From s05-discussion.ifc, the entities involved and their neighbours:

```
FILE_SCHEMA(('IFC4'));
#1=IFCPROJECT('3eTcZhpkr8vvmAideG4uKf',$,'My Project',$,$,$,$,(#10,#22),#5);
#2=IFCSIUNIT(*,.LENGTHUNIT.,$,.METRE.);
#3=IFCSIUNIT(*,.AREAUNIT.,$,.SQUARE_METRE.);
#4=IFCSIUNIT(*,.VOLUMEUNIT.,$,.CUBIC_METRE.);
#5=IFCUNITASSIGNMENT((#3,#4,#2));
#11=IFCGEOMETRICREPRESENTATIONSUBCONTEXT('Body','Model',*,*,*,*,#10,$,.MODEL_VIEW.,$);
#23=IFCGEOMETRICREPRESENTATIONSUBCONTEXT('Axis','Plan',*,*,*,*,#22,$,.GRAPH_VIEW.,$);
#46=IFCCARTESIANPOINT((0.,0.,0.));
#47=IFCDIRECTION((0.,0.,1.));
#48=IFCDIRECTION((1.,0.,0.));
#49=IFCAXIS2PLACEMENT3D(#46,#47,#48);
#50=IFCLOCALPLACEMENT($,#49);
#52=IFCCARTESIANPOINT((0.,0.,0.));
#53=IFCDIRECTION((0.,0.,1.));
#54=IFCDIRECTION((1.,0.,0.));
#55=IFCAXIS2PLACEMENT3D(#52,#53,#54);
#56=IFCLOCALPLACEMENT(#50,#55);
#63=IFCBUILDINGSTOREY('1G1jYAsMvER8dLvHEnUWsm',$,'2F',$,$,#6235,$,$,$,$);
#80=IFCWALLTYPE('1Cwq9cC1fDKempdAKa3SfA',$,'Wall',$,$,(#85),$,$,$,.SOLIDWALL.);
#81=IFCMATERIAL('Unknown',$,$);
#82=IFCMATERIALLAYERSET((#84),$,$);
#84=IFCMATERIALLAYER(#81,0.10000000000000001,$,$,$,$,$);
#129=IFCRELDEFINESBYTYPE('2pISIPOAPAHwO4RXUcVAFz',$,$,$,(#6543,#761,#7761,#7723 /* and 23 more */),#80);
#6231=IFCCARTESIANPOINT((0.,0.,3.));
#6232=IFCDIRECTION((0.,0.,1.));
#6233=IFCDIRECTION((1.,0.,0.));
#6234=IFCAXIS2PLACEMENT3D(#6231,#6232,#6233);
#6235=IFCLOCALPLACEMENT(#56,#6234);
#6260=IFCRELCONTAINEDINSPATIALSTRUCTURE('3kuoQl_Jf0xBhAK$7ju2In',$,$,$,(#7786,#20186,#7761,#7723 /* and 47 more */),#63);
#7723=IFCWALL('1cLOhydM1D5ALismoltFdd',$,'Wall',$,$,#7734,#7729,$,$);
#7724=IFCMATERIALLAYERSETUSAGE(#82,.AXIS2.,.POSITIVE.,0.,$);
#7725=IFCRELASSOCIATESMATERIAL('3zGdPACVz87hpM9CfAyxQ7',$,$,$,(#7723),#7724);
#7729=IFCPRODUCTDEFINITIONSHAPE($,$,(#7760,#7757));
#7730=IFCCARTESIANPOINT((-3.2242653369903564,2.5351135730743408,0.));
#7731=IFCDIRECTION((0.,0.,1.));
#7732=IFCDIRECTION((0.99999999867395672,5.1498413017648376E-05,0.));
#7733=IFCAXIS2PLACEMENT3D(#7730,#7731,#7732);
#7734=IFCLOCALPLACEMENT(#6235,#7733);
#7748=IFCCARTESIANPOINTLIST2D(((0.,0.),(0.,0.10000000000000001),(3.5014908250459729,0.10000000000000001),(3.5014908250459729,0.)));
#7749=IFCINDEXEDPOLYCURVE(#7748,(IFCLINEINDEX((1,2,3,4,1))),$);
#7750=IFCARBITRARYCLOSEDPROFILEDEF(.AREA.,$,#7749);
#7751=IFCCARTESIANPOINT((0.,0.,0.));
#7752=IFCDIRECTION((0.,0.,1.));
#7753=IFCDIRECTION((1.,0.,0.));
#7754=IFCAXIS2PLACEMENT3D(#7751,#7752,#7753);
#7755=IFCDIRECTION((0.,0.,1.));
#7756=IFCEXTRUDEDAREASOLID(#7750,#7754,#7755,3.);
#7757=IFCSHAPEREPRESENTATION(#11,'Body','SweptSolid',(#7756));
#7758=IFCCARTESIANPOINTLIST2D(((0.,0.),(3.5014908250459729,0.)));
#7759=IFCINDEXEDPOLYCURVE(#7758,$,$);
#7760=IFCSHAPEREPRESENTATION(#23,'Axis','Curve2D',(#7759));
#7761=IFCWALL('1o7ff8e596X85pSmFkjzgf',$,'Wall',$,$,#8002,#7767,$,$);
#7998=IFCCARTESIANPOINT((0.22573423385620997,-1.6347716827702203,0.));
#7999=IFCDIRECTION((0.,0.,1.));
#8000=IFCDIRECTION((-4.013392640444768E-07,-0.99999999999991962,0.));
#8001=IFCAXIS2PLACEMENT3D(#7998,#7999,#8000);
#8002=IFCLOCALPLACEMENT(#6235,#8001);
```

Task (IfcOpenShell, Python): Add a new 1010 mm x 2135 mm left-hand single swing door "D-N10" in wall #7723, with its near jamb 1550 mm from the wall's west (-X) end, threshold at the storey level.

```python
import numpy as np
import ifcopenshell
import ifcopenshell.api.feature
import ifcopenshell.api.geometry
import ifcopenshell.api.root
import ifcopenshell.api.spatial
import ifcopenshell.geom
import ifcopenshell.util.element
import ifcopenshell.util.placement
import ifcopenshell.util.representation
import ifcopenshell.util.shape
import ifcopenshell.util.unit

model = ifcopenshell.open("s05-discussion.ifc")
unit_scale = ifcopenshell.util.unit.calculate_unit_scale(model)
settings = ifcopenshell.geom.settings()


def volume(element):
    """Net volume in cubic metres, openings subtracted."""
    shape = ifcopenshell.geom.create_shape(settings, element)
    return ifcopenshell.util.shape.get_volume(shape.geometry)


wall = model.by_guid("1cLOhydM1D5ALismoltFdd")
storey = ifcopenshell.util.element.get_container(wall, ifc_class="IfcBuildingStorey")
context = ifcopenshell.util.representation.get_context(model, "Model", "Body", "MODEL_VIEW")
before = volume(wall)

width, height, from_end, sill = 1.01, 2.135, 1.55, 0.0  # metres

# The wall runs along its own X axis, and the end named is its -X end.
wall_shape = ifcopenshell.geom.create_shape(settings, wall)
x, y, z = ifcopenshell.util.shape.get_vertices(wall_shape.geometry).T
start = x.min() + from_end
face, thickness = float(y.min()), float(y.max() - y.min())
wall_matrix = ifcopenshell.util.placement.get_local_placement(wall.ObjectPlacement)
level = ifcopenshell.util.placement.get_local_placement(storey.ObjectPlacement)[2, 3]


def in_wall(x, y):
    """Placement at x, y metres in the wall's axes, at sill height."""
    matrix = wall_matrix.copy()
    matrix[:, 3] = wall_matrix @ np.array([x / unit_scale, y / unit_scale, 0.0, 1.0])
    matrix[2, 3] = level + sill / unit_scale
    return matrix


# Opening: a box that overshoots both wall faces by 50 mm.
opening = ifcopenshell.api.root.create_entity(model, ifc_class="IfcOpeningElement", predefined_type="OPENING")
box = ifcopenshell.api.geometry.add_wall_representation(
    model, context=context, length=width, height=height, thickness=thickness + 0.1
)
ifcopenshell.api.geometry.assign_representation(model, product=opening, representation=box)
ifcopenshell.api.geometry.edit_object_placement(model, product=opening, matrix=in_wall(start, face - 0.05), is_si=False)
ifcopenshell.api.feature.add_feature(model, feature=opening, element=wall)

door = ifcopenshell.api.root.create_entity(model, ifc_class="IfcDoor", name="D-N10", predefined_type="DOOR")
door.OverallWidth, door.OverallHeight = width / unit_scale, height / unit_scale
door.OperationType = "SINGLE_SWING_LEFT"
body = ifcopenshell.api.geometry.add_door_representation(
    model,
    context=context,
    overall_width=door.OverallWidth,
    overall_height=door.OverallHeight,
    operation_type="SINGLE_SWING_LEFT",
    lining_properties={"LiningDepth": thickness / unit_scale, "ThresholdDepth": thickness / unit_scale},
)
ifcopenshell.api.geometry.assign_representation(model, product=door, representation=body)
ifcopenshell.api.spatial.assign_container(model, products=[door], relating_structure=storey)
ifcopenshell.api.feature.add_filling(model, opening=opening, element=door)

# The lining spans the wall, so the door starts at the wall face.
ifcopenshell.api.geometry.edit_object_placement(model, product=door, matrix=in_wall(start, face), is_si=False)

after = volume(wall)

print(f"wall volume {before:.3f} -> {after:.3f} m3")

model.write("s05-discussion_rev.ifc")
```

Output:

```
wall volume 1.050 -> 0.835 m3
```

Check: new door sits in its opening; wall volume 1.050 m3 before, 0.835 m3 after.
